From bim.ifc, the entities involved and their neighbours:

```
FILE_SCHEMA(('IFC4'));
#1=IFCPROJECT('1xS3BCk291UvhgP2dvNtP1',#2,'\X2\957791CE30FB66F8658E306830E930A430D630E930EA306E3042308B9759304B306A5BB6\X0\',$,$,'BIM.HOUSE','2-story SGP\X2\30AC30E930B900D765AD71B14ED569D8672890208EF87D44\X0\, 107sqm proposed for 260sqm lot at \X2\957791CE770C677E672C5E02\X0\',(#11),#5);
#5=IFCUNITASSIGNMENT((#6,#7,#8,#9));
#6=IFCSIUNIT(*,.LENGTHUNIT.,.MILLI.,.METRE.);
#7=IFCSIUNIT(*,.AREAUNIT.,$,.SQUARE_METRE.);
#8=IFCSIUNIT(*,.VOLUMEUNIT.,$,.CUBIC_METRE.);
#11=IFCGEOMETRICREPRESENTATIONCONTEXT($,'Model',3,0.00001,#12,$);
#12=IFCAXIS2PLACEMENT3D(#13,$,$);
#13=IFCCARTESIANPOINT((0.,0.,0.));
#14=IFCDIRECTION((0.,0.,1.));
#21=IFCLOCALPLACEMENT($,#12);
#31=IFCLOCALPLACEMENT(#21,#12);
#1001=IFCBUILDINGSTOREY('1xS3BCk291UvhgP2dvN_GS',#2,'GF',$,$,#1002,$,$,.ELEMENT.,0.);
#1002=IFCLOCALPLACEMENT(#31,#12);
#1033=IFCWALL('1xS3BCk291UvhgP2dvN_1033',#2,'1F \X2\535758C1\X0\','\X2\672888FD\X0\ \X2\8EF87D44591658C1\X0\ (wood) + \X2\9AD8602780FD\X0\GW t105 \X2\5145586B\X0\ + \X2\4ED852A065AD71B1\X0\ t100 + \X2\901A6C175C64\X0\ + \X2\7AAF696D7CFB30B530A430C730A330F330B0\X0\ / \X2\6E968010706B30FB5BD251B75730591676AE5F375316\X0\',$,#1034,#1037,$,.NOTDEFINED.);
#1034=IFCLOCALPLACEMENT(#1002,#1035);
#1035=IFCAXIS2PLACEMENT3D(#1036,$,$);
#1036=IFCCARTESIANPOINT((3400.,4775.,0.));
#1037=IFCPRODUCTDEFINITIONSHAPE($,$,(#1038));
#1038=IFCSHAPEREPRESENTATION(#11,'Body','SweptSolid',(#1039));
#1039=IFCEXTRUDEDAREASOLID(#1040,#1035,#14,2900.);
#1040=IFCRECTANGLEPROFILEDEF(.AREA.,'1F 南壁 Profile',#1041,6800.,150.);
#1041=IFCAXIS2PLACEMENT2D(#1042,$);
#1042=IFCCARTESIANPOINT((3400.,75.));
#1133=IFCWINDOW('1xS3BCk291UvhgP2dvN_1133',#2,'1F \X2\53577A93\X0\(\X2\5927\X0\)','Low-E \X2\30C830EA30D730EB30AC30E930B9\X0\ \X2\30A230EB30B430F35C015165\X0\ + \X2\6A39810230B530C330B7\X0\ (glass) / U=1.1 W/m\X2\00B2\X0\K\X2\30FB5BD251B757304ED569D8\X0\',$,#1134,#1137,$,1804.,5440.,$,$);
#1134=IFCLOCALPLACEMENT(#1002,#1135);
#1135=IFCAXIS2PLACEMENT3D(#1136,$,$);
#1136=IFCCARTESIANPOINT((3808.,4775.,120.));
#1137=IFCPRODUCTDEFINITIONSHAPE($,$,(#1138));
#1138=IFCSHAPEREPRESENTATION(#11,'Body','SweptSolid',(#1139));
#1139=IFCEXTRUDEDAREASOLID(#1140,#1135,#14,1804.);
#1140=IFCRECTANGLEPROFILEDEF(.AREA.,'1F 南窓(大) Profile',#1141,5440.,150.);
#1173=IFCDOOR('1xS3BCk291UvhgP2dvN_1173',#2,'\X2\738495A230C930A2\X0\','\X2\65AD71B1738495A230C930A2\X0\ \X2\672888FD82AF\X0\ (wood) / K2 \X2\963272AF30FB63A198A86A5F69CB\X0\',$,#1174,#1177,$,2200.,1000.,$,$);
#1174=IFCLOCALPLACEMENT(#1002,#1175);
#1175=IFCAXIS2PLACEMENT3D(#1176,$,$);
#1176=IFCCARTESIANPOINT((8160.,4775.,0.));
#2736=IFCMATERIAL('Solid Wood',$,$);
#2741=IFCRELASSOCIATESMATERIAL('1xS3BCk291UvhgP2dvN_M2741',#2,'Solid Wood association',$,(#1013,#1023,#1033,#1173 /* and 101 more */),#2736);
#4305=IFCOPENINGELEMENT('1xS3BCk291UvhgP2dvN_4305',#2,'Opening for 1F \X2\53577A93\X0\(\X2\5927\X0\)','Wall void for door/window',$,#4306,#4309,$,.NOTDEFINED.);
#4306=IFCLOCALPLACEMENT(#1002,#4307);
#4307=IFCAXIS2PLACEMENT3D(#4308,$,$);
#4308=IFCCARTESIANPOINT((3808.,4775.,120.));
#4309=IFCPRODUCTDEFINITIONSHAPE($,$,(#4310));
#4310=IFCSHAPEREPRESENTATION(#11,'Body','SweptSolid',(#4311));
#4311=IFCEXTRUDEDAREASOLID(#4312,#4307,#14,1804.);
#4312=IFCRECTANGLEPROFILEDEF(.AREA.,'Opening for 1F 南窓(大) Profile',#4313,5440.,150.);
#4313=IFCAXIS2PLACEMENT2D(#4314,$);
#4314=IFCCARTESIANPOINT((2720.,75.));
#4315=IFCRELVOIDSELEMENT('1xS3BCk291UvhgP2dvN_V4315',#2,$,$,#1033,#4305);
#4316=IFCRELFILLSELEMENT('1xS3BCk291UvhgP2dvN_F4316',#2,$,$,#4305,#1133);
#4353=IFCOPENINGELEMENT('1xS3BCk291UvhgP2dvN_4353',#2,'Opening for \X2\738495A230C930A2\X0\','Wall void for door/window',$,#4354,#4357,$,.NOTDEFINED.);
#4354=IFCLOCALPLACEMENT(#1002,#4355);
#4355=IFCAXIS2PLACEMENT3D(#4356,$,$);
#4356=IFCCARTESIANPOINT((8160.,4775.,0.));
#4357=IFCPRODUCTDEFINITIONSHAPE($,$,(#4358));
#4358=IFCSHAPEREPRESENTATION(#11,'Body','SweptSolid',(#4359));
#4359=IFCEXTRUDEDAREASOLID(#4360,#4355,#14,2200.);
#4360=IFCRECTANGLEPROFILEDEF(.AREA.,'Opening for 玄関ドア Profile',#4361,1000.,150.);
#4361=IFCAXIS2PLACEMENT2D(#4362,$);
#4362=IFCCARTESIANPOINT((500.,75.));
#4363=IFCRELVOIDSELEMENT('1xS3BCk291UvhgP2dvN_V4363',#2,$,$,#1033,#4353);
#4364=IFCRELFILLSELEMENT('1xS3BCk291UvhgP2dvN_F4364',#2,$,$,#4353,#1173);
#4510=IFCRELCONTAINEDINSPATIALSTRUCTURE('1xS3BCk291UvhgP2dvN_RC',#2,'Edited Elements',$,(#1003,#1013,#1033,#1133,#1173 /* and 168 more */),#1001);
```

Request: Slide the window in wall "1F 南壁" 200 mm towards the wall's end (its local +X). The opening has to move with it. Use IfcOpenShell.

```python
import ifcopenshell
import ifcopenshell.api.geometry
import ifcopenshell.util.placement

model = ifcopenshell.open("bim.ifc")

window = model.by_guid("1xS3BCk291UvhgP2dvN_1133")
opening = window.FillsVoids[0].RelatingOpeningElement
wall = opening.VoidsElements[0].RelatingBuildingElement

wall_matrix = ifcopenshell.util.placement.get_local_placement(wall.ObjectPlacement)
shift = wall_matrix[:3, 0] * 200.0
before = ifcopenshell.util.placement.get_local_placement(window.ObjectPlacement)[:3, 3].copy()

# The window is not placed relative to its opening, so move both.
for product in (opening, window):
    matrix = ifcopenshell.util.placement.get_local_placement(product.ObjectPlacement)
    matrix[:3, 3] += shift
    ifcopenshell.api.geometry.edit_object_placement(model, product=product, matrix=matrix, is_si=False)

after = ifcopenshell.util.placement.get_local_placement(window.ObjectPlacement)[:3, 3]
print("window moved by", (after - before).round(3) + 0.0)

model.write("bim_rev.ifc")
```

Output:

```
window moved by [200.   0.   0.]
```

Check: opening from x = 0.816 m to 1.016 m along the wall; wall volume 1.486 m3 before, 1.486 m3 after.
